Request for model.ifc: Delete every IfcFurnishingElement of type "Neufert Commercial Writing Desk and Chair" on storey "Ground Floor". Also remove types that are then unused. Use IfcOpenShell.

First a look at what the model holds.

```python
import ifcopenshell
import ifcopenshell.util.element

model = ifcopenshell.open("model.ifc")
print(model.schema)
storey = next(s for s in model.by_type("IfcBuildingStorey") if s.Name == "Ground Floor")
furniture = [e for e in ifcopenshell.util.element.get_decomposition(storey) if e.is_a("IfcFurnishingElement")]
seen = {}
for e in furniture:
    element_type = ifcopenshell.util.element.get_type(e)
    name = element_type.Name if element_type not in (None, e) else None
    seen[name] = seen.get(name, 0) + 1
for name, count in sorted(seen.items(), key=str):
    print(count, "x", name)
```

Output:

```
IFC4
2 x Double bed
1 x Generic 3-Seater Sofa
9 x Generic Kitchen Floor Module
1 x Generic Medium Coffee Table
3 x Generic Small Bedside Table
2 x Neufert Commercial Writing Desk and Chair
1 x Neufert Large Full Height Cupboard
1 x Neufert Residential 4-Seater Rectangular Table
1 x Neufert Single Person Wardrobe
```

```python
import ifcopenshell
import ifcopenshell.api.root
import ifcopenshell.util.element

model = ifcopenshell.open("model.ifc")

storey = next(s for s in model.by_type("IfcBuildingStorey") if s.Name == "Ground Floor")
furniture = [e for e in ifcopenshell.util.element.get_decomposition(storey) if e.is_a("IfcFurnishingElement")]
targets = [e for e in furniture if (t := ifcopenshell.util.element.get_type(e)) not in (None, e) and t.Name == "Neufert Commercial Writing Desk and Chair"]
types = {ifcopenshell.util.element.get_type(e) for e in targets} - {None, *targets}

for e in targets:
    ifcopenshell.api.root.remove_product(model, product=e)
print(len(targets), "removed")

unused = [t for t in types if not ifcopenshell.util.element.get_types(t)]
for t in unused:
    ifcopenshell.api.root.remove_product(model, product=t)
print(len(unused), "unused types removed")

model.write("model_v2.ifc")
```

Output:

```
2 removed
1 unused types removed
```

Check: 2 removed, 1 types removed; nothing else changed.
